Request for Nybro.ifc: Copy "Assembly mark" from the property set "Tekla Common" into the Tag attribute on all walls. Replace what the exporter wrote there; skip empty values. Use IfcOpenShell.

First a look at what the model holds.

```python
import ifcopenshell
import ifcopenshell.util.element

model = ifcopenshell.open("Nybro.ifc")
print(model.schema)
walls = model.by_type("IfcWall")
print(len(walls), "walls")
for e in walls[:8]:
    source = ifcopenshell.util.element.get_pset(e, "Tekla Common", "Assembly mark")
    target = e.Tag
    print(e.id(), repr(source), repr(target), sep=" | ")
```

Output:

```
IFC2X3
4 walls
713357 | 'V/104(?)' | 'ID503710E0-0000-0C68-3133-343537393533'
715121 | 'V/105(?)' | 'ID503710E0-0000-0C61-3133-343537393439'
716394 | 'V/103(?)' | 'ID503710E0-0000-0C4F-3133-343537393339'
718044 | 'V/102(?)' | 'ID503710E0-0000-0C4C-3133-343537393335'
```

```python
import ifcopenshell
import ifcopenshell.util.element

model = ifcopenshell.open("Nybro.ifc")

count = 0
for e in model.by_type("IfcWall"):
    value = ifcopenshell.util.element.get_pset(e, "Tekla Common", "Assembly mark")
    current = e.Tag
    if not value or not value.strip() or current == value:
        continue
    e.Tag = value
    count += 1

print(count, "walls updated")

model.write("Nybro_v2.ifc")
```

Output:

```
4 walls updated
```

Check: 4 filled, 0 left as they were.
